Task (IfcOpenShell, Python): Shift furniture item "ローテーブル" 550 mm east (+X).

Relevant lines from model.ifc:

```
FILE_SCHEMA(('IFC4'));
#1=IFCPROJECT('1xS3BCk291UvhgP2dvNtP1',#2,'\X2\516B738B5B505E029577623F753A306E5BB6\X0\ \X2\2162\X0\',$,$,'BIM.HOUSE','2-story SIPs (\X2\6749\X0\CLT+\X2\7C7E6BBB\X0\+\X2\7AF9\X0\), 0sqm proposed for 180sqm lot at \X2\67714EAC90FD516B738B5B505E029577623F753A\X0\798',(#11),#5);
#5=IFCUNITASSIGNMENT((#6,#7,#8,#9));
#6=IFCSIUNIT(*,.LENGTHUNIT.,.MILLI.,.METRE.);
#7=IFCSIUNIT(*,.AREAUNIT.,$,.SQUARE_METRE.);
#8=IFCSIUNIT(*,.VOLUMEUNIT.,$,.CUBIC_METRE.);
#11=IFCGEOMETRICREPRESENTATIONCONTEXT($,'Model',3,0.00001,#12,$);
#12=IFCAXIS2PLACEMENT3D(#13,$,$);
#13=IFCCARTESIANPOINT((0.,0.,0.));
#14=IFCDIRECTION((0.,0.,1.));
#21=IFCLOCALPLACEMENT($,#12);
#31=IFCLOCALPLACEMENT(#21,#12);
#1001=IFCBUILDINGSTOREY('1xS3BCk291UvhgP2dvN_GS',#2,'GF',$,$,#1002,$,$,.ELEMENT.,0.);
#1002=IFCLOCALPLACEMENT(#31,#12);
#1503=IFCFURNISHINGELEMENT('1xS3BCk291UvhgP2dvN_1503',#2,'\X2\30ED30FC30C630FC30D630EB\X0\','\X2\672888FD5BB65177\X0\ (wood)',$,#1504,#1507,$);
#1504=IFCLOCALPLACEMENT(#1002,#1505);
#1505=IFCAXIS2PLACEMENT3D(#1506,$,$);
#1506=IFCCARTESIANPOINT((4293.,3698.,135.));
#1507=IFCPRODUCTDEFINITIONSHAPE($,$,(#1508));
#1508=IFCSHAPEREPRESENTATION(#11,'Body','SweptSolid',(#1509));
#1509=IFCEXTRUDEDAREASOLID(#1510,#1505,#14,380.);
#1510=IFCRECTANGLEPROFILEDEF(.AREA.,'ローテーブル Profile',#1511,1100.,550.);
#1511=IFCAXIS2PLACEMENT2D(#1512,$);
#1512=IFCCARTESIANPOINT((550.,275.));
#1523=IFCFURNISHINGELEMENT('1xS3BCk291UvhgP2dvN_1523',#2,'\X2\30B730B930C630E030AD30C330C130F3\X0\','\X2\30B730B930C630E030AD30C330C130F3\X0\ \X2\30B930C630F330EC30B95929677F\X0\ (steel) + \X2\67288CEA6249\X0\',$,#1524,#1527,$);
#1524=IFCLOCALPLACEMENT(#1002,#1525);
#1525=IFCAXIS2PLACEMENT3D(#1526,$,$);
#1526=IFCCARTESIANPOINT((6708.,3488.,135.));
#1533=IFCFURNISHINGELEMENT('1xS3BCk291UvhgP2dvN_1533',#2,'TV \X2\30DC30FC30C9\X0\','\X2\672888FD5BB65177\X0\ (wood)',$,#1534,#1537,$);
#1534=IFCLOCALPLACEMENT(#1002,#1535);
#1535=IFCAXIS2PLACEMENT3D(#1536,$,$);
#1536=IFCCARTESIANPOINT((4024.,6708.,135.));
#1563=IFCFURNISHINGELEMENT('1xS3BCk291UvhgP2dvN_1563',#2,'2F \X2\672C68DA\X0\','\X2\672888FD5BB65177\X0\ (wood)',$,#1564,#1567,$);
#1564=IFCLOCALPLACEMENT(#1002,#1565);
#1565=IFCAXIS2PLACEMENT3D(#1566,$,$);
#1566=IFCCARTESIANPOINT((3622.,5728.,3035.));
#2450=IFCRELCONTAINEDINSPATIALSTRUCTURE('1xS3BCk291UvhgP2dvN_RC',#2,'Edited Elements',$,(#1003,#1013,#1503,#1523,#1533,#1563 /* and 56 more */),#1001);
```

```python
import ifcopenshell
import ifcopenshell.api.geometry
import ifcopenshell.util.placement
import ifcopenshell.util.unit

model = ifcopenshell.open("model.ifc")
unit_scale = ifcopenshell.util.unit.calculate_unit_scale(model)

item = model.by_guid("1xS3BCk291UvhgP2dvN_1503")
matrix = ifcopenshell.util.placement.get_local_placement(item.ObjectPlacement)
matrix[0, 3] += 0.55 / unit_scale
ifcopenshell.api.geometry.edit_object_placement(model, product=item, matrix=matrix, is_si=False)

print(ifcopenshell.util.placement.get_local_placement(item.ObjectPlacement).round(3) + 0.0)

model.write("model_rev.ifc")
```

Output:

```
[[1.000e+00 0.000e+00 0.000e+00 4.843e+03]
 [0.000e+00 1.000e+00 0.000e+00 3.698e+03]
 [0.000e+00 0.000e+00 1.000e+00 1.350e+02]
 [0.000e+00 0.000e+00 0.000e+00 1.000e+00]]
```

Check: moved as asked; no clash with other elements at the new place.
